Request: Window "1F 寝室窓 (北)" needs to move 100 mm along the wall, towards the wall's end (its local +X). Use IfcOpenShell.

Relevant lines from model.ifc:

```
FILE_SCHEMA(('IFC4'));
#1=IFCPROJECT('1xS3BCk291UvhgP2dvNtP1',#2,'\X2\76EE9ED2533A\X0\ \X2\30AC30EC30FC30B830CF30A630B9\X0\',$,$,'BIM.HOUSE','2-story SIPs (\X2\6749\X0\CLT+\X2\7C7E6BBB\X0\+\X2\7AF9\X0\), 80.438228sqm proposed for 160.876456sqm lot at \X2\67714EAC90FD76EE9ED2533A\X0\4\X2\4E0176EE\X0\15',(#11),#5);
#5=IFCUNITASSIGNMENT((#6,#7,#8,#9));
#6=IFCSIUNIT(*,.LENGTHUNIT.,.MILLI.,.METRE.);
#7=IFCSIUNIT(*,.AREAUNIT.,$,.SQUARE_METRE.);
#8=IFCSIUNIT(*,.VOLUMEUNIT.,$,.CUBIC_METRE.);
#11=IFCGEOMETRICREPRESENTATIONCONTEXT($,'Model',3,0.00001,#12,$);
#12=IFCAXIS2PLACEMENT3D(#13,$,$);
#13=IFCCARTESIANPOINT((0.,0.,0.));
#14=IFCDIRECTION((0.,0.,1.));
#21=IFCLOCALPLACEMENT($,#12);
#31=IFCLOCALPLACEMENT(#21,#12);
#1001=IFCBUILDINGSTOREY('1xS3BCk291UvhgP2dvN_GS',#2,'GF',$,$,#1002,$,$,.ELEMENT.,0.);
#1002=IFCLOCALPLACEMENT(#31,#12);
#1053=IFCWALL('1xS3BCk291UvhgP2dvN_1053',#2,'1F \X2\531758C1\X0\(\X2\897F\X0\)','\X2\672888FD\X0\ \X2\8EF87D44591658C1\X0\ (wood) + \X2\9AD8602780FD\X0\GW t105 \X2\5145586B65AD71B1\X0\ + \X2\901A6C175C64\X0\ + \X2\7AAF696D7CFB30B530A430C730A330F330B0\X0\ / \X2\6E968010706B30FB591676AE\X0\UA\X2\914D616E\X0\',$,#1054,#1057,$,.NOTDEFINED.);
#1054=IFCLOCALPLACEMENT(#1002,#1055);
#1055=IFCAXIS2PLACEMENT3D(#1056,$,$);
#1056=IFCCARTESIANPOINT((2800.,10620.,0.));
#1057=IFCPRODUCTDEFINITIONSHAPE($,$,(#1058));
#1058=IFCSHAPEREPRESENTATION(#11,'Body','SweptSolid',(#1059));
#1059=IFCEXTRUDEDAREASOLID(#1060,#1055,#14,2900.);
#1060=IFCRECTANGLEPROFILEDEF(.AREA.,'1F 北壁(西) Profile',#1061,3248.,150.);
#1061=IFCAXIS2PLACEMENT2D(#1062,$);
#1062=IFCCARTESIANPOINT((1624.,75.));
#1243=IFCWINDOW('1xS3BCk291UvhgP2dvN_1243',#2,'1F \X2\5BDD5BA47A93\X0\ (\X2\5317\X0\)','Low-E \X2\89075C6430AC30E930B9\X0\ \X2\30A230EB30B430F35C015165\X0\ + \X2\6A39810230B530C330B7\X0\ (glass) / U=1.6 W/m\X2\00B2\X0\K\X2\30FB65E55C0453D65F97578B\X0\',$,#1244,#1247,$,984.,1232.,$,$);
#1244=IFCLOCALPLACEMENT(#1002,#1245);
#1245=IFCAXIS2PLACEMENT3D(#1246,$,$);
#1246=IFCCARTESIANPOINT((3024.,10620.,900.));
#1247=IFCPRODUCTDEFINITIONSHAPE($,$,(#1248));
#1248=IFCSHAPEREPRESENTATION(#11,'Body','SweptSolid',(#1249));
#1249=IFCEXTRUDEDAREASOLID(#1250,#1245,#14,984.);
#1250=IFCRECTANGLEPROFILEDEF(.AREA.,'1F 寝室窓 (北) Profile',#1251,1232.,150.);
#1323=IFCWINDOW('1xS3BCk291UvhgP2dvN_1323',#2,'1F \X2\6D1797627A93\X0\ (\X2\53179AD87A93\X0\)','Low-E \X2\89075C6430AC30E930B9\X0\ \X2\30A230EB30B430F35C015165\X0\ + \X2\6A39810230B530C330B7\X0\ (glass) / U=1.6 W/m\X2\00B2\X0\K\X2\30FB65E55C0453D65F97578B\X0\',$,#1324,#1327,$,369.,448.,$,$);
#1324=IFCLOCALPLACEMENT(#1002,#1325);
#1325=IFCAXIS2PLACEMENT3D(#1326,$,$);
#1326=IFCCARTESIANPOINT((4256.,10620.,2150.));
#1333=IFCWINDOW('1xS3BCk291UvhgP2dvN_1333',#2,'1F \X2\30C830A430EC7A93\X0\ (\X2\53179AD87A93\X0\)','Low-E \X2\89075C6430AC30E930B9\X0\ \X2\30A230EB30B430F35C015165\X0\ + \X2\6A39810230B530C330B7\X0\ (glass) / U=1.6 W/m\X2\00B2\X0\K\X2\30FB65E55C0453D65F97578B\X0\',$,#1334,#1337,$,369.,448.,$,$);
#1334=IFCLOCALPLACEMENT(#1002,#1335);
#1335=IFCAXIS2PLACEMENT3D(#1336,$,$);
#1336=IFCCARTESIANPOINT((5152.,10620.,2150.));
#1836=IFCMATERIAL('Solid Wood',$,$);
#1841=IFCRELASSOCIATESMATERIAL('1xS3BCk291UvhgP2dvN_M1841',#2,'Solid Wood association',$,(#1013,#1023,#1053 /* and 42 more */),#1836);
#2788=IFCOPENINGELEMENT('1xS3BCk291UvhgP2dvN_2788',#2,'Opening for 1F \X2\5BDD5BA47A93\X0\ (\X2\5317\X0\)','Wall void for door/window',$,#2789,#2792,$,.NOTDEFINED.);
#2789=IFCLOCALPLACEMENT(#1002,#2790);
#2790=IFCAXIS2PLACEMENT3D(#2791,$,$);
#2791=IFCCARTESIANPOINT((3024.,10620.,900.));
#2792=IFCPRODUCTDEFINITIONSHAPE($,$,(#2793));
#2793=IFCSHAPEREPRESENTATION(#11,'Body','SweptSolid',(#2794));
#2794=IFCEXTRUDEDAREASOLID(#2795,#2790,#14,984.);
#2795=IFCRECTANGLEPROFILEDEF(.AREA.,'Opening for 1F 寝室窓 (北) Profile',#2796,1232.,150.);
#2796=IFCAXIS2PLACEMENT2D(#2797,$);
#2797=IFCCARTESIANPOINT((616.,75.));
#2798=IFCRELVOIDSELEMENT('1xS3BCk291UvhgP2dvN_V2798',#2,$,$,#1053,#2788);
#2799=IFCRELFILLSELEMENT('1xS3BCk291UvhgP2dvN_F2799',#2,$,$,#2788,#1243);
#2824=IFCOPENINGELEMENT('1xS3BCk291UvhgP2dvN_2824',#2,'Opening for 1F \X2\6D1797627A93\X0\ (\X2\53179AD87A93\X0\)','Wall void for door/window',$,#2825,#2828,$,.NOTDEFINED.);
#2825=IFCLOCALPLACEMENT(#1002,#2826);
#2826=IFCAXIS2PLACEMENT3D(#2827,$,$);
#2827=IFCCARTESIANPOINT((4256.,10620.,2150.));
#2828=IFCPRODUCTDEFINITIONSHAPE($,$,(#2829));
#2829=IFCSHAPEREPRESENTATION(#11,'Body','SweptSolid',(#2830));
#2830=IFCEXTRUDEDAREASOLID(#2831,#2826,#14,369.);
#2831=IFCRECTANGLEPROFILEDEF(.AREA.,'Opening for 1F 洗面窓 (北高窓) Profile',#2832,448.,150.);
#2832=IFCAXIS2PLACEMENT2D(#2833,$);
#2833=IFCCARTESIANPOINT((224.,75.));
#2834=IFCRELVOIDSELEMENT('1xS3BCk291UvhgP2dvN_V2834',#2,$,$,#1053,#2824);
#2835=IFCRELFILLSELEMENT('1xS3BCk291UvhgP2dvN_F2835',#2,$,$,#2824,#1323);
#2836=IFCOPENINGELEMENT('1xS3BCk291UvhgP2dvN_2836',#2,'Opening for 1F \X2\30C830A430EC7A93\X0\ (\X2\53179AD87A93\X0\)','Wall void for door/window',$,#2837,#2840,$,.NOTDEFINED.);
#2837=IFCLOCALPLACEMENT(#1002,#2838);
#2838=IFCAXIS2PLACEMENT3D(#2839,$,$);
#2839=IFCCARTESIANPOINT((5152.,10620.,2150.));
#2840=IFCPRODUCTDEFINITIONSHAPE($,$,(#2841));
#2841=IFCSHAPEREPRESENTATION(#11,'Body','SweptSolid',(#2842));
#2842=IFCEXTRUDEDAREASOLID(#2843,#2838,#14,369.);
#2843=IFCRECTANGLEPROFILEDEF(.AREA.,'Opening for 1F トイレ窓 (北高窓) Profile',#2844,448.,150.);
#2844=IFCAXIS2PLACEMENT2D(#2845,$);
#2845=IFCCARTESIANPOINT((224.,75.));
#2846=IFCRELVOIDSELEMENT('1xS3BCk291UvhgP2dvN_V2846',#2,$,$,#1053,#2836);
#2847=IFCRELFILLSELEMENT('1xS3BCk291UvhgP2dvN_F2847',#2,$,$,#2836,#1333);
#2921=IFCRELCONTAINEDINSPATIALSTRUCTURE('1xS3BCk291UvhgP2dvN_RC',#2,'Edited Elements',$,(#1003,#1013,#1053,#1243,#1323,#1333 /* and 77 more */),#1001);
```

```python
import ifcopenshell
import ifcopenshell.api.geometry
import ifcopenshell.util.placement
import ifcopenshell.util.unit

model = ifcopenshell.open("model.ifc")
unit_scale = ifcopenshell.util.unit.calculate_unit_scale(model)

window = model.by_id(1243)
opening = window.FillsVoids[0].RelatingOpeningElement
wall = opening.VoidsElements[0].RelatingBuildingElement

wall_matrix = ifcopenshell.util.placement.get_local_placement(wall.ObjectPlacement)
shift = wall_matrix[:3, 0] * 0.1 / unit_scale
before = ifcopenshell.util.placement.get_local_placement(window.ObjectPlacement)[:3, 3].copy()

# The window is not placed relative to its opening, so move both.
for product in (opening, window):
    matrix = ifcopenshell.util.placement.get_local_placement(product.ObjectPlacement)
    matrix[:3, 3] += shift
    ifcopenshell.api.geometry.edit_object_placement(model, product=product, matrix=matrix, is_si=False)

after = ifcopenshell.util.placement.get_local_placement(window.ObjectPlacement)[:3, 3]
print("window moved by", (after - before).round(3) + 0.0)

model.write("model_v2.ifc")
```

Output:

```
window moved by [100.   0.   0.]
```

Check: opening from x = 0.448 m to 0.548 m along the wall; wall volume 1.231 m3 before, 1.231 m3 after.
